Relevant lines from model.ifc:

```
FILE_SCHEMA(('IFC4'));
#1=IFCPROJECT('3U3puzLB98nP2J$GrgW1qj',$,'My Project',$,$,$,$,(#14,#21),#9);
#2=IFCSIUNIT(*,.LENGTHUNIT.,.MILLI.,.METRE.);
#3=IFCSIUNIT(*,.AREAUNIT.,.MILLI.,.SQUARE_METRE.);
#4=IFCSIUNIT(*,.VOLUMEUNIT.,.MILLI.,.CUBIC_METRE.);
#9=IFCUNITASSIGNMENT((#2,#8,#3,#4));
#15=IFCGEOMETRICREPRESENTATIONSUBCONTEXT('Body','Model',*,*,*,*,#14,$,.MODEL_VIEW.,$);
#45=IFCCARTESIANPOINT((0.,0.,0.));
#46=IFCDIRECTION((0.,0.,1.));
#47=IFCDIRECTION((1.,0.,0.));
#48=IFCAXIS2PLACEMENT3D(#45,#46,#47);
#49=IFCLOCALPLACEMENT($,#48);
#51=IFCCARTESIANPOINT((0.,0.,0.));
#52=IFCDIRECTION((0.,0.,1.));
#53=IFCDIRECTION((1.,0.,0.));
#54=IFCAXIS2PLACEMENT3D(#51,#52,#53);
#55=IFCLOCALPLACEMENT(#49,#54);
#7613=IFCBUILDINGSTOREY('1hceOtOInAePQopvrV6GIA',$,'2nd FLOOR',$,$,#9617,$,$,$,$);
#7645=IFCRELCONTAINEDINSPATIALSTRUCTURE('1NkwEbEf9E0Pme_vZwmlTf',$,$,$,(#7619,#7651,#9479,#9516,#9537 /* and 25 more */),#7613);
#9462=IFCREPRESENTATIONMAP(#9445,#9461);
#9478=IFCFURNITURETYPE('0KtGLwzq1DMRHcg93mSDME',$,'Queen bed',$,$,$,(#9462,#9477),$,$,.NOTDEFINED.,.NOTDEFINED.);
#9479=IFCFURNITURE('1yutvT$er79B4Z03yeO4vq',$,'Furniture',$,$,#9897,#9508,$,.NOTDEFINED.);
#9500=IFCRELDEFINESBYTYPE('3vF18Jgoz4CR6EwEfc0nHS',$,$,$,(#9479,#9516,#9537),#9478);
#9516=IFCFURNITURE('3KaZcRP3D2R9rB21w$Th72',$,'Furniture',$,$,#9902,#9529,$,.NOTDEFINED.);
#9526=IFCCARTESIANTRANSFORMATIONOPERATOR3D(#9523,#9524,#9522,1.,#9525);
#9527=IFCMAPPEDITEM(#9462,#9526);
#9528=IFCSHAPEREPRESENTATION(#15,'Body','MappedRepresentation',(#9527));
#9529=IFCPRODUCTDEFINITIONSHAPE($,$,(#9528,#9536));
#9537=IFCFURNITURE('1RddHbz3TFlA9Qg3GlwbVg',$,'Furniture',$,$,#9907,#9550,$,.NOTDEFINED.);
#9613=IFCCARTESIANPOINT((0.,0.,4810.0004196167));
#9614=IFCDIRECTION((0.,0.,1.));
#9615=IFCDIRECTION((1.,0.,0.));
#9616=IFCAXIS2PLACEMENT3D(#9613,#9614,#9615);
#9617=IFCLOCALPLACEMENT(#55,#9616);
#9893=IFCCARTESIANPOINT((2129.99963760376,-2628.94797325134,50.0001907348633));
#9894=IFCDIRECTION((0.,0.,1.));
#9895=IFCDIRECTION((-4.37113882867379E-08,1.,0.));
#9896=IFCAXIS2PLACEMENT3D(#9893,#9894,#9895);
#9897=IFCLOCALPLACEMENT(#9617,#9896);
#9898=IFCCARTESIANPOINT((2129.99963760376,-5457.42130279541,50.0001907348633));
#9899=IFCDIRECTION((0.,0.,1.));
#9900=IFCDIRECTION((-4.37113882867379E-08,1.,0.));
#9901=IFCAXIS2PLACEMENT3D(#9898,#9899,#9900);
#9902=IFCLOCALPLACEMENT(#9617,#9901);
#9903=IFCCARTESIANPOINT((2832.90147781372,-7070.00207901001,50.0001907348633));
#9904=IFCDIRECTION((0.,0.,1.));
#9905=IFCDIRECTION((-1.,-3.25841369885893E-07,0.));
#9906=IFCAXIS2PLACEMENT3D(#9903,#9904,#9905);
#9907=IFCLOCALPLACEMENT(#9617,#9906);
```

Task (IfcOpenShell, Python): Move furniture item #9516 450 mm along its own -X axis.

```python
import ifcopenshell
import ifcopenshell.api.geometry
import ifcopenshell.util.placement
import ifcopenshell.util.unit

model = ifcopenshell.open("model.ifc")
unit_scale = ifcopenshell.util.unit.calculate_unit_scale(model)

item = model.by_guid("3KaZcRP3D2R9rB21w$Th72")
matrix = ifcopenshell.util.placement.get_local_placement(item.ObjectPlacement)
matrix[:3, 3] -= matrix[:3, 0] * 0.45 / unit_scale
ifcopenshell.api.geometry.edit_object_placement(model, product=item, matrix=matrix, is_si=False)

print(ifcopenshell.util.placement.get_local_placement(item.ObjectPlacement).round(3) + 0.0)

model.write("model_edited.ifc")
```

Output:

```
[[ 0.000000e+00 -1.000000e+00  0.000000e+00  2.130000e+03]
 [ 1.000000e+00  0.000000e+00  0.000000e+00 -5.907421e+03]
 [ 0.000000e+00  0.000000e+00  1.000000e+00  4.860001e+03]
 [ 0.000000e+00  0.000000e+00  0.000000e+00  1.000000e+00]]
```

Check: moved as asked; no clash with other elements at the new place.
